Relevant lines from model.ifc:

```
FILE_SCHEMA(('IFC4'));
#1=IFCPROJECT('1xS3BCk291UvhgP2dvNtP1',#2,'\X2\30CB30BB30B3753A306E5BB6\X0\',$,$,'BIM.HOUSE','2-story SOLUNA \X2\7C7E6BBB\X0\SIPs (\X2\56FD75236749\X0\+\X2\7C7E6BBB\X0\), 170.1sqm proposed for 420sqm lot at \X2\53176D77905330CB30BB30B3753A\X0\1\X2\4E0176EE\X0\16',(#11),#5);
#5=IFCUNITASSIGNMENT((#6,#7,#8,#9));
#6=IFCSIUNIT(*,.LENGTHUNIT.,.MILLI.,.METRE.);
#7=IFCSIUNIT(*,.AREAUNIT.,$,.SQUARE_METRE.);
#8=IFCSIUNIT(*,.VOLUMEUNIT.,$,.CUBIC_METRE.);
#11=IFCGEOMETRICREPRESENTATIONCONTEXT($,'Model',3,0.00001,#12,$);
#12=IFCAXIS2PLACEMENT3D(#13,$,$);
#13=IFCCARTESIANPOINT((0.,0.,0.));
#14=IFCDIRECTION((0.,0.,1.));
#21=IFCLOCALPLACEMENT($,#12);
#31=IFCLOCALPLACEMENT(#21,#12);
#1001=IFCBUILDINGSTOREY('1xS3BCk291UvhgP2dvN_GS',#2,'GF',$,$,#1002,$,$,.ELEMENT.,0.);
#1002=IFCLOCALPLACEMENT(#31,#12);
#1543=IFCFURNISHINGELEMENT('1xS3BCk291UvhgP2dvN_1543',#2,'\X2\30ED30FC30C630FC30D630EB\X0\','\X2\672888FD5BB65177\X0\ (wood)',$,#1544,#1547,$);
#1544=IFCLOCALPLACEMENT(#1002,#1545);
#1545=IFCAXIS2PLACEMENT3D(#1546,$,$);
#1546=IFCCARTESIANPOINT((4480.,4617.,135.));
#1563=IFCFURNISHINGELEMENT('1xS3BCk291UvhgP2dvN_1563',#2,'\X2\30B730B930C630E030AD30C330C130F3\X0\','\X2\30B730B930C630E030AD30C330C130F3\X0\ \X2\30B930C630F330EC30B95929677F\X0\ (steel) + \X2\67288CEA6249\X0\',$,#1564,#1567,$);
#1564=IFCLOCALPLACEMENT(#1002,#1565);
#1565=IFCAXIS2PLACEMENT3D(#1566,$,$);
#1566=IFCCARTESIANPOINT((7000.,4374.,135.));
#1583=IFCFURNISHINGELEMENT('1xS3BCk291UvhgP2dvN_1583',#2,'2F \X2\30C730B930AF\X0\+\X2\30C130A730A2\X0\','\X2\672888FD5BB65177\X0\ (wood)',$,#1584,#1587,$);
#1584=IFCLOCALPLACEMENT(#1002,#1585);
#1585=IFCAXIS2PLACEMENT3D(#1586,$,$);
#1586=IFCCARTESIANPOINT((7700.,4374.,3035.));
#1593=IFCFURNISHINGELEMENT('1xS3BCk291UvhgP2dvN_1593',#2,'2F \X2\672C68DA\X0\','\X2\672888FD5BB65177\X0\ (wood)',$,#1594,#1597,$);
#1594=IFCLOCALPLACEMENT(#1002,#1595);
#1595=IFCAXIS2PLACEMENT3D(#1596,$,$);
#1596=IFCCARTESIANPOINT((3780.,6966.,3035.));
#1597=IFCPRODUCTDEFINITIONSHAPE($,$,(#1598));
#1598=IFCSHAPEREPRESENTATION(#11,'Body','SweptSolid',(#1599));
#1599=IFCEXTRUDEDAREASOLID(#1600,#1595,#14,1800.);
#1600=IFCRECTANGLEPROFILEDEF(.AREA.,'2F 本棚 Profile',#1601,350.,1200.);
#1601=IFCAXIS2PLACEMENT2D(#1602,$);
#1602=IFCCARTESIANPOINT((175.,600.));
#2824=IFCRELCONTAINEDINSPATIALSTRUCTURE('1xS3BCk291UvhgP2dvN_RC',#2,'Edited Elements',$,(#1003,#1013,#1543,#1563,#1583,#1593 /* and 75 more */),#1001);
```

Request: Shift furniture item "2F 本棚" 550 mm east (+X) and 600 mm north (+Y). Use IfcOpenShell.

```python
import ifcopenshell
import ifcopenshell.api.geometry
import ifcopenshell.util.placement

model = ifcopenshell.open("model.ifc")

item = model.by_guid("1xS3BCk291UvhgP2dvN_1593")
matrix = ifcopenshell.util.placement.get_local_placement(item.ObjectPlacement)
matrix[0, 3] += 550.0
matrix[1, 3] += 600.0
ifcopenshell.api.geometry.edit_object_placement(model, product=item, matrix=matrix, is_si=False)

print(ifcopenshell.util.placement.get_local_placement(item.ObjectPlacement).round(3) + 0.0)

model.write("model_rev.ifc")
```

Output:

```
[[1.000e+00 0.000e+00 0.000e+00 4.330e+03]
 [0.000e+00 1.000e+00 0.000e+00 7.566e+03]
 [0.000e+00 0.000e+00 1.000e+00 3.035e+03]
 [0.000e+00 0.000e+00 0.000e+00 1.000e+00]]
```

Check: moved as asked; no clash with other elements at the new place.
